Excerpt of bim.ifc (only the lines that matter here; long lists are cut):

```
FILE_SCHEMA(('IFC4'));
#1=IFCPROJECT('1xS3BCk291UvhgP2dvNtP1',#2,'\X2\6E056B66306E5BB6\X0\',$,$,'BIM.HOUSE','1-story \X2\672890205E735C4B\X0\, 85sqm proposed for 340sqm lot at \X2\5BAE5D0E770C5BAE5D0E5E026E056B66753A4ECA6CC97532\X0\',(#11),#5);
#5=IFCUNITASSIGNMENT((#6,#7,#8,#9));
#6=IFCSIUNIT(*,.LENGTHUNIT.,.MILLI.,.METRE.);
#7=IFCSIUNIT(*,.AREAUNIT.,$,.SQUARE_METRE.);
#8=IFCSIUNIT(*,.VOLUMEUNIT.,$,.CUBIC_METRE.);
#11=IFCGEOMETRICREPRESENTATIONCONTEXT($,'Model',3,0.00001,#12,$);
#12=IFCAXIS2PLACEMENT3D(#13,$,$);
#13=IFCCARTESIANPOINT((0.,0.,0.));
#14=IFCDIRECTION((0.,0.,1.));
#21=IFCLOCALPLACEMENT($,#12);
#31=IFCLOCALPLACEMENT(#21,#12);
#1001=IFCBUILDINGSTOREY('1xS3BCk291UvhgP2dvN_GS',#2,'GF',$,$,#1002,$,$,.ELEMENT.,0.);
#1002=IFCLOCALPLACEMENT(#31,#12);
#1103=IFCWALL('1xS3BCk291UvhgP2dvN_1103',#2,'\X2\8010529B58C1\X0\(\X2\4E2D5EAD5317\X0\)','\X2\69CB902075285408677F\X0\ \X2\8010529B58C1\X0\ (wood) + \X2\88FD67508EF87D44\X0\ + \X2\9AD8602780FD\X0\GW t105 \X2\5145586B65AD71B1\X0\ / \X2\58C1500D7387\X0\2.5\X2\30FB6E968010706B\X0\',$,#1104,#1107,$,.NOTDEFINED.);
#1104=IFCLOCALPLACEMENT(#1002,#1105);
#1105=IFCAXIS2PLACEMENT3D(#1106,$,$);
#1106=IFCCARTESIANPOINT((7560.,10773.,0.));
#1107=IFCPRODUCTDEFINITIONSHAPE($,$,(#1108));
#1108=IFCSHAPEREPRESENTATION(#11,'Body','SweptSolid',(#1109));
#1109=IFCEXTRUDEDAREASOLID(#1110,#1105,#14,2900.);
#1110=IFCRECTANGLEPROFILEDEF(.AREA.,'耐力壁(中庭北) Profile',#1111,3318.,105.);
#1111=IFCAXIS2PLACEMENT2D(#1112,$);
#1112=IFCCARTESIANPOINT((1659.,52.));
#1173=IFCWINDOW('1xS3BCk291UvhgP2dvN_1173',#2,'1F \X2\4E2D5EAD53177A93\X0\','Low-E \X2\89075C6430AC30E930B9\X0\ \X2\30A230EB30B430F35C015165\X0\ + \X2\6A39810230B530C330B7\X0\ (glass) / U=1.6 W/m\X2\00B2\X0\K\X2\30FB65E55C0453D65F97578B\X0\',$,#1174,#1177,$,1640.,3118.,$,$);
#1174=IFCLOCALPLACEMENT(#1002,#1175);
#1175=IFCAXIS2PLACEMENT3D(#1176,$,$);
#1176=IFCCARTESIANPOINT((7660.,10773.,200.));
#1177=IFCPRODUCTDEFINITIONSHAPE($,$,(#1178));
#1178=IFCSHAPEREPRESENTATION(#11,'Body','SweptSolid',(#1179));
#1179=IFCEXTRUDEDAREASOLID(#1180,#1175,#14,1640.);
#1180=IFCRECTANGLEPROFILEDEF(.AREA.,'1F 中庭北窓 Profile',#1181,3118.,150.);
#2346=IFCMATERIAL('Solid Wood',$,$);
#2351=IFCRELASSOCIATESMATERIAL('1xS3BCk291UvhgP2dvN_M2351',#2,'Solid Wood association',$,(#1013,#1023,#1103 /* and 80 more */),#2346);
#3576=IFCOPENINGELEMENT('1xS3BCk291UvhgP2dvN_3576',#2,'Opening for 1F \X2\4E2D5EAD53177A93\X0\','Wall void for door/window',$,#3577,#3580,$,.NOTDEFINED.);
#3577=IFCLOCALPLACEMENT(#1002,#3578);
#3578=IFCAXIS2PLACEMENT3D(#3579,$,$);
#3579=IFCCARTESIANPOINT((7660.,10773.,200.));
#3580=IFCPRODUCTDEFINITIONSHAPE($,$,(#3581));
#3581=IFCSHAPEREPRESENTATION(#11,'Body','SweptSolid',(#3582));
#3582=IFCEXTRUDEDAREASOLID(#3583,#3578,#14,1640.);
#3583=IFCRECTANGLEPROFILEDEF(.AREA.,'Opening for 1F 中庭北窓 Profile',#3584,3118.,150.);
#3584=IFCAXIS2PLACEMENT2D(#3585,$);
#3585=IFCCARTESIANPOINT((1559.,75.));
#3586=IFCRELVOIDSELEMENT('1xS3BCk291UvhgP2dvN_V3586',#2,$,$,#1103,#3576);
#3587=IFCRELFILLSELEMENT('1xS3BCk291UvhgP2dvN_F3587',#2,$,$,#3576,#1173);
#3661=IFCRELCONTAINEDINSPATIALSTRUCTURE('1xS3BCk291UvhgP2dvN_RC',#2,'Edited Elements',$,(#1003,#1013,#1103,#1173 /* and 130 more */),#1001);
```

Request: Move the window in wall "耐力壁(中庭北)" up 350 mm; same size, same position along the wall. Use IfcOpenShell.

```python
import numpy as np
import ifcopenshell
import ifcopenshell.api.geometry
import ifcopenshell.util.placement
import ifcopenshell.util.unit

model = ifcopenshell.open("bim.ifc")
unit_scale = ifcopenshell.util.unit.calculate_unit_scale(model)

window = model.by_id(1173)
opening = window.FillsVoids[0].RelatingOpeningElement
dz = 0.35 / unit_scale

shift = np.array([0.0, 0.0, dz])
# The window is not placed relative to its opening, so move both.
for product in (opening, window):
    matrix = ifcopenshell.util.placement.get_local_placement(product.ObjectPlacement)
    matrix[:3, 3] += shift
    ifcopenshell.api.geometry.edit_object_placement(model, product=product, matrix=matrix, is_si=False)

print(f"moved by {dz * unit_scale:+.3f} m")

model.write("bim-out.ifc")
```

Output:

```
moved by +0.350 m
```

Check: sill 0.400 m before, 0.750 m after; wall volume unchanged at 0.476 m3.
